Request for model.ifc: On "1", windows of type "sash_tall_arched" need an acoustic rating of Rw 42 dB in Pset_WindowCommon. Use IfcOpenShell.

First a look at what the model holds.

```python
import ifcopenshell
import ifcopenshell.util.element

model = ifcopenshell.open("model.ifc")
print(model.schema)
storey = next(s for s in model.by_type("IfcBuildingStorey") if s.Name == "1")
windows = [e for e in ifcopenshell.util.element.get_decomposition(storey) if e.is_a("IfcWindow")]
seen = {}
for e in windows:
    element_type = ifcopenshell.util.element.get_type(e)
    key = (element_type.Name if element_type != e and element_type else None, ifcopenshell.util.element.get_pset(e, "Pset_WindowCommon", "AcousticRating"))
    seen[key] = seen.get(key, 0) + 1
for (name, value), count in sorted(seen.items(), key=str):
    print(count, "x", name, "|", value)
```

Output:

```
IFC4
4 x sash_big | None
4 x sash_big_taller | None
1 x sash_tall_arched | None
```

```python
import ifcopenshell
import ifcopenshell.api.pset
import ifcopenshell.util.element

model = ifcopenshell.open("model.ifc")

storey = next(s for s in model.by_type("IfcBuildingStorey") if s.Name == "1")
windows = [e for e in ifcopenshell.util.element.get_decomposition(storey) if e.is_a("IfcWindow")]

count = 0
for e in windows:
    element_type = ifcopenshell.util.element.get_type(e)
    if element_type in (None, e) or element_type.Name != "sash_tall_arched":
        continue
    # add_pset returns the element's existing set when there is one.
    pset = ifcopenshell.api.pset.add_pset(model, product=e, name="Pset_WindowCommon")
    ifcopenshell.api.pset.edit_pset(model, pset=pset, properties={"AcousticRating": "Rw 42 dB"})
    count += 1

print(count, "windows updated")

model.write("model_v2.ifc")
```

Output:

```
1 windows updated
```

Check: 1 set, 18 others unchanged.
